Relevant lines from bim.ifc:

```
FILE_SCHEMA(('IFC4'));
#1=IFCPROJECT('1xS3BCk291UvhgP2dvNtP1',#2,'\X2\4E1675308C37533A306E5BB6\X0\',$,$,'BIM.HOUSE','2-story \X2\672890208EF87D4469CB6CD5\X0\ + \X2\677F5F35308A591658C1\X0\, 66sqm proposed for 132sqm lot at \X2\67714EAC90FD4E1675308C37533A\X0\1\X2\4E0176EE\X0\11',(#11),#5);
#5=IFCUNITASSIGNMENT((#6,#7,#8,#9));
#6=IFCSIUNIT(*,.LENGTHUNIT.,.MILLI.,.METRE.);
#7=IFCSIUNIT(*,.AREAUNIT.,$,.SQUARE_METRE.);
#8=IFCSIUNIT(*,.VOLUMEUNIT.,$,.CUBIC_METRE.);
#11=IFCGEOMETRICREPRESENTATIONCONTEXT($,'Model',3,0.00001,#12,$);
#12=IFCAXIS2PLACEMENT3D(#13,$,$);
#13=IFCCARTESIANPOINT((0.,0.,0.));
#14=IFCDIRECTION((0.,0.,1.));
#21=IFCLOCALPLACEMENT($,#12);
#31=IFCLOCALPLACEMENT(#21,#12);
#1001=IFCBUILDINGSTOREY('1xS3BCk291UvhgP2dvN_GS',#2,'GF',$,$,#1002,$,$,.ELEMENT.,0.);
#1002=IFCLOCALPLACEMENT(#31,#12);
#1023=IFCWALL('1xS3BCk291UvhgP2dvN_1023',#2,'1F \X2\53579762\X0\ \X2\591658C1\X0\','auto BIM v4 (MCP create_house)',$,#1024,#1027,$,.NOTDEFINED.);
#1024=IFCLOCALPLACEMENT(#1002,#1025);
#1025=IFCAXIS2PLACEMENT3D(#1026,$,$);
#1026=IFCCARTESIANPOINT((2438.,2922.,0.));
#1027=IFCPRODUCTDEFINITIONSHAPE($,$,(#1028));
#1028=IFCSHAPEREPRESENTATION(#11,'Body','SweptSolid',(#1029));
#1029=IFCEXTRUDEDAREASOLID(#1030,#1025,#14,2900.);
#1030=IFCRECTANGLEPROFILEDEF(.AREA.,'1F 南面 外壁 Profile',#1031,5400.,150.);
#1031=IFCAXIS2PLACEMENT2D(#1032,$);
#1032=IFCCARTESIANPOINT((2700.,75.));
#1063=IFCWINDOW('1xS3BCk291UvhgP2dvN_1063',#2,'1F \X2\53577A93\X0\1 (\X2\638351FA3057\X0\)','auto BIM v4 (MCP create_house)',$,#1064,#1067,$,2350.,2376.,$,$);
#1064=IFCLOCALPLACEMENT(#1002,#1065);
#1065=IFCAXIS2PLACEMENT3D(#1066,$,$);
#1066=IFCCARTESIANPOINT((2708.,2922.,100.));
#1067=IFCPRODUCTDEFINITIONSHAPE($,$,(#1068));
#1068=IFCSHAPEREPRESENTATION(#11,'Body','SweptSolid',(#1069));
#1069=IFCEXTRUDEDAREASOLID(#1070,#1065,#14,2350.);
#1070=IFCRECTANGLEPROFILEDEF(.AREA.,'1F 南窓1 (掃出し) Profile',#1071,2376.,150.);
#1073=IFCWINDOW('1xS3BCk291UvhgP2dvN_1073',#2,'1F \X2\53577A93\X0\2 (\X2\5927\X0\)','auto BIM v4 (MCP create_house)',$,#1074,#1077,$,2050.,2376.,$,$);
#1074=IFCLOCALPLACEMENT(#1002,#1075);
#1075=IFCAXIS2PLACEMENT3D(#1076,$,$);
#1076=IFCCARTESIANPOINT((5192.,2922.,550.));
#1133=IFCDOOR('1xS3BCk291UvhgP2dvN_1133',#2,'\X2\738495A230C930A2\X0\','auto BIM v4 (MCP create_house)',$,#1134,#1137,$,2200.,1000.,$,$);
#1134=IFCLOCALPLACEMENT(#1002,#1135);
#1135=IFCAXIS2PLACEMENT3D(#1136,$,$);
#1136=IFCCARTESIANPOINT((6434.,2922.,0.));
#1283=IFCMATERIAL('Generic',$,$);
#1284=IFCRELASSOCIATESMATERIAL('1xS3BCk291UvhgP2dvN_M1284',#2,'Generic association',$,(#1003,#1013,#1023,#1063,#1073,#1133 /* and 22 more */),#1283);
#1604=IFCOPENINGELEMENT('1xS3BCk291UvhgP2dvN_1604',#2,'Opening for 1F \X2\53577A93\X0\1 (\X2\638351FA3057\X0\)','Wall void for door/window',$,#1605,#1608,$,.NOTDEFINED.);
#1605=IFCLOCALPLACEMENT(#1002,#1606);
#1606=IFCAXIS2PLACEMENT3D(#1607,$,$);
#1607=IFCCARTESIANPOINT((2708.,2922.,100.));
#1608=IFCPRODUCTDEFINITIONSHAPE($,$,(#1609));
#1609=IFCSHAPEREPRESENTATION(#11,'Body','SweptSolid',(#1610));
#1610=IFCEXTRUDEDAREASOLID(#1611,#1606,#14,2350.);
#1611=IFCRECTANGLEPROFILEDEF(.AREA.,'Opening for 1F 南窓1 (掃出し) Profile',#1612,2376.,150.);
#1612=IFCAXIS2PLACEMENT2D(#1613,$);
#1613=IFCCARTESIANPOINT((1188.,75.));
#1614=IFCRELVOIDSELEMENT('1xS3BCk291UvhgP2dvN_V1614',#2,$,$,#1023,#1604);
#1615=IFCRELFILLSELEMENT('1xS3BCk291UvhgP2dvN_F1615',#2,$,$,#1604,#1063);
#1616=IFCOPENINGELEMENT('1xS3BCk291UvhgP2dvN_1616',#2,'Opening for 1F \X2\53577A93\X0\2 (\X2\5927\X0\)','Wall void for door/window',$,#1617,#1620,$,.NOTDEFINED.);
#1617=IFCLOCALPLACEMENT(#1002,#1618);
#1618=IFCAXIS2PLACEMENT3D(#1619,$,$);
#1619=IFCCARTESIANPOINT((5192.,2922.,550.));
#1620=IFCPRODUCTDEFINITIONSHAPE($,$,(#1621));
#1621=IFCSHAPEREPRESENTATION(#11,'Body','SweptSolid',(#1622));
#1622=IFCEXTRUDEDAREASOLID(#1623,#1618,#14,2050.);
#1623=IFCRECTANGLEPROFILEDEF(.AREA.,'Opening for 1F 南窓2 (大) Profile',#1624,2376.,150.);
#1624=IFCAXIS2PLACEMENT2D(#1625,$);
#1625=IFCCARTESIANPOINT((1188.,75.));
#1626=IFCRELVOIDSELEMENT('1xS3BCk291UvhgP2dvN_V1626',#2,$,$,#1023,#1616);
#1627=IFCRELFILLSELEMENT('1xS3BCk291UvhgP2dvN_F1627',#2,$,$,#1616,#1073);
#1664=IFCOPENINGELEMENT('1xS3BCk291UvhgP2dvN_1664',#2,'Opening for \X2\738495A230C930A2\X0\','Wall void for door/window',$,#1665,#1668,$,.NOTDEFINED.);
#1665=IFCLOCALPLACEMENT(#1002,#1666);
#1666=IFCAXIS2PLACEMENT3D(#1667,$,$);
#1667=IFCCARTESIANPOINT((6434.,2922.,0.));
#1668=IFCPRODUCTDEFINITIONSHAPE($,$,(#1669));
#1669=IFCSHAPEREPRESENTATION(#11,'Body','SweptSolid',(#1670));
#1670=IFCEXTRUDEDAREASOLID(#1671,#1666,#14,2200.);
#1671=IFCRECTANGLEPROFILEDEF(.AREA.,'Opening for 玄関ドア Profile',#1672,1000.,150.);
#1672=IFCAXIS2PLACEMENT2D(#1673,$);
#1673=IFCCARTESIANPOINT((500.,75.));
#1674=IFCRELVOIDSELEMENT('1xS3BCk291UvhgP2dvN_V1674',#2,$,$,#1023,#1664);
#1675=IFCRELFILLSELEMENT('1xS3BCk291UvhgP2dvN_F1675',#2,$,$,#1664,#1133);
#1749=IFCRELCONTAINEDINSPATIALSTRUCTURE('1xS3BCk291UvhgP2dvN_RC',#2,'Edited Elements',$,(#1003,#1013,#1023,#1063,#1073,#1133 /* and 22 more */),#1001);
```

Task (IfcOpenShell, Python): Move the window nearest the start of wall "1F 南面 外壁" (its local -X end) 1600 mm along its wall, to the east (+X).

```python
import ifcopenshell
import ifcopenshell.api.geometry
import ifcopenshell.util.placement
import ifcopenshell.util.unit

model = ifcopenshell.open("bim.ifc")
unit_scale = ifcopenshell.util.unit.calculate_unit_scale(model)

window = model.by_guid("1xS3BCk291UvhgP2dvN_1063")
opening = window.FillsVoids[0].RelatingOpeningElement
wall = opening.VoidsElements[0].RelatingBuildingElement

wall_matrix = ifcopenshell.util.placement.get_local_placement(wall.ObjectPlacement)
shift = wall_matrix[:3, 0] * 1.6 / unit_scale
before = ifcopenshell.util.placement.get_local_placement(window.ObjectPlacement)[:3, 3].copy()

# The window is not placed relative to its opening, so move both.
for product in (opening, window):
    matrix = ifcopenshell.util.placement.get_local_placement(product.ObjectPlacement)
    matrix[:3, 3] += shift
    ifcopenshell.api.geometry.edit_object_placement(model, product=product, matrix=matrix, is_si=False)

after = ifcopenshell.util.placement.get_local_placement(window.ObjectPlacement)[:3, 3]
print("window moved by", (after - before).round(3) + 0.0)

model.write("bim_rev.ifc")
```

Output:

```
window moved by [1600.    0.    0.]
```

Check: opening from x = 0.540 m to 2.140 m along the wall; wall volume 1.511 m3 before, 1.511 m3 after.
